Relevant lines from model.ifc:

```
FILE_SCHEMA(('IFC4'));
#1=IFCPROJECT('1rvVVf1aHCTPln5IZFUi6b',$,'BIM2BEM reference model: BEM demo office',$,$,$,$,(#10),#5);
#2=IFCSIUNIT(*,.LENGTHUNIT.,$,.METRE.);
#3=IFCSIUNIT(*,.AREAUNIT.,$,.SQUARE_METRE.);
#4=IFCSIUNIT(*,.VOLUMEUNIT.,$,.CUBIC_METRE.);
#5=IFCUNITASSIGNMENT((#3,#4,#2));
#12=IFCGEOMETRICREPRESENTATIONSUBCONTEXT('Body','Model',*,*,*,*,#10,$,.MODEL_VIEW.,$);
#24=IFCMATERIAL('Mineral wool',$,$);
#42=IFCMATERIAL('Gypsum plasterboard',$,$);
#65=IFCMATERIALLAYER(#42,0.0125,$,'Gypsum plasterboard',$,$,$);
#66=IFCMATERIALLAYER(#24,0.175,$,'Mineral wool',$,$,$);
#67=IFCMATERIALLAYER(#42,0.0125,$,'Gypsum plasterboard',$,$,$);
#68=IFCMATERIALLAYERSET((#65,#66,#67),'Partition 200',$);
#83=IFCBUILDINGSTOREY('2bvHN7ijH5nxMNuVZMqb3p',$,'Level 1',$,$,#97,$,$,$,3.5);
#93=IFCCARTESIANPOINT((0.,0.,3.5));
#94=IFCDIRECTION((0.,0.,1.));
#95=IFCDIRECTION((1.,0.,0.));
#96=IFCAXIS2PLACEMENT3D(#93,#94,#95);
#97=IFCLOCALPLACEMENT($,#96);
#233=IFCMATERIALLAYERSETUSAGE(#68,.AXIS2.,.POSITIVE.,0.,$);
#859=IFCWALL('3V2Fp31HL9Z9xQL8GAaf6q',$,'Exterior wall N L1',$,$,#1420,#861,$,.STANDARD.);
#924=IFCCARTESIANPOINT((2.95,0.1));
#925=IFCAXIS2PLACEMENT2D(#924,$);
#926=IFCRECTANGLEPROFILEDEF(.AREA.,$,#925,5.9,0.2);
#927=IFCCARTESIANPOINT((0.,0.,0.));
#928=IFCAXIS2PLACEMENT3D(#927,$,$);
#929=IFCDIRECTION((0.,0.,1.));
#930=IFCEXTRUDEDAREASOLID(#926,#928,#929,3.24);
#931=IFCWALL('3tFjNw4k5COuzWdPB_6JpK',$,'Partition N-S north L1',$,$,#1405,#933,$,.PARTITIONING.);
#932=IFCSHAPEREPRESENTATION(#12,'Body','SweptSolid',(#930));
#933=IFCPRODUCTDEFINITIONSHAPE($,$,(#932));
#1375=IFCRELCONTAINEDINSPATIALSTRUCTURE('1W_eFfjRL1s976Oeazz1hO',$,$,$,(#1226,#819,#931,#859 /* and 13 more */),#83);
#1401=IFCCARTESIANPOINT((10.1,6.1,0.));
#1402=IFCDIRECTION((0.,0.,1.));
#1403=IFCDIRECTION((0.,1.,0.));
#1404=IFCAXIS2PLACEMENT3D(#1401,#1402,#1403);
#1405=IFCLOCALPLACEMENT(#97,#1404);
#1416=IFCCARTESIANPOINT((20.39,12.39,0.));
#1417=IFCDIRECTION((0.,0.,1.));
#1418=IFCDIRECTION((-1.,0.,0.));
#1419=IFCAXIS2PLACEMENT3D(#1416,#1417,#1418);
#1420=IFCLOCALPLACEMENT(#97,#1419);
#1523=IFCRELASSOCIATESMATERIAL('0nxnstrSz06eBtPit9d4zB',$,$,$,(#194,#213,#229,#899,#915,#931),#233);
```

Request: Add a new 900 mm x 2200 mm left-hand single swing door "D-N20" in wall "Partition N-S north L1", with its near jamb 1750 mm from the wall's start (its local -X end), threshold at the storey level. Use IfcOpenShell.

```python
import numpy as np
import ifcopenshell
import ifcopenshell.api.feature
import ifcopenshell.api.geometry
import ifcopenshell.api.root
import ifcopenshell.api.spatial
import ifcopenshell.geom
import ifcopenshell.util.element
import ifcopenshell.util.placement
import ifcopenshell.util.representation
import ifcopenshell.util.shape
import ifcopenshell.util.unit

model = ifcopenshell.open("model.ifc")
unit_scale = ifcopenshell.util.unit.calculate_unit_scale(model)
settings = ifcopenshell.geom.settings()


def volume(element):
    """Net volume in cubic metres, openings subtracted."""
    shape = ifcopenshell.geom.create_shape(settings, element)
    return ifcopenshell.util.shape.get_volume(shape.geometry)


wall = model.by_guid("3tFjNw4k5COuzWdPB_6JpK")
storey = ifcopenshell.util.element.get_container(wall, ifc_class="IfcBuildingStorey")
context = ifcopenshell.util.representation.get_context(model, "Model", "Body", "MODEL_VIEW")
before = volume(wall)

width, height, from_end, sill = 0.9, 2.2, 1.75, 0.0  # metres

# The wall runs along its own X axis, and the end named is its -X end.
wall_shape = ifcopenshell.geom.create_shape(settings, wall)
x, y, z = ifcopenshell.util.shape.get_vertices(wall_shape.geometry).T
start = x.min() + from_end
face, thickness = float(y.min()), float(y.max() - y.min())
wall_matrix = ifcopenshell.util.placement.get_local_placement(wall.ObjectPlacement)
level = ifcopenshell.util.placement.get_local_placement(storey.ObjectPlacement)[2, 3]


def in_wall(x, y):
    """Placement at x, y metres in the wall's axes, at sill height."""
    matrix = wall_matrix.copy()
    matrix[:, 3] = wall_matrix @ np.array([x / unit_scale, y / unit_scale, 0.0, 1.0])
    matrix[2, 3] = level + sill / unit_scale
    return matrix


# Opening: a box that overshoots both wall faces by 50 mm.
opening = ifcopenshell.api.root.create_entity(model, ifc_class="IfcOpeningElement", predefined_type="OPENING")
box = ifcopenshell.api.geometry.add_wall_representation(
    model, context=context, length=width, height=height, thickness=thickness + 0.1
)
ifcopenshell.api.geometry.assign_representation(model, product=opening, representation=box)
ifcopenshell.api.geometry.edit_object_placement(model, product=opening, matrix=in_wall(start, face - 0.05), is_si=False)
ifcopenshell.api.feature.add_feature(model, feature=opening, element=wall)

door = ifcopenshell.api.root.create_entity(model, ifc_class="IfcDoor", name="D-N20", predefined_type="DOOR")
door.OverallWidth, door.OverallHeight = width / unit_scale, height / unit_scale
door.OperationType = "SINGLE_SWING_LEFT"
body = ifcopenshell.api.geometry.add_door_representation(
    model,
    context=context,
    overall_width=door.OverallWidth,
    overall_height=door.OverallHeight,
    operation_type="SINGLE_SWING_LEFT",
    lining_properties={"LiningDepth": thickness / unit_scale, "ThresholdDepth": thickness / unit_scale},
)
ifcopenshell.api.geometry.assign_representation(model, product=door, representation=body)
ifcopenshell.api.spatial.assign_container(model, products=[door], relating_structure=storey)
ifcopenshell.api.feature.add_filling(model, opening=opening, element=door)

# The lining spans the wall, so the door starts at the wall face.
ifcopenshell.api.geometry.edit_object_placement(model, product=door, matrix=in_wall(start, face), is_si=False)

after = volume(wall)

print(f"wall volume {before:.3f} -> {after:.3f} m3")

model.write("model-out.ifc")
```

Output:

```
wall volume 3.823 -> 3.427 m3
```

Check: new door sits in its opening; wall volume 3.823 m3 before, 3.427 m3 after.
